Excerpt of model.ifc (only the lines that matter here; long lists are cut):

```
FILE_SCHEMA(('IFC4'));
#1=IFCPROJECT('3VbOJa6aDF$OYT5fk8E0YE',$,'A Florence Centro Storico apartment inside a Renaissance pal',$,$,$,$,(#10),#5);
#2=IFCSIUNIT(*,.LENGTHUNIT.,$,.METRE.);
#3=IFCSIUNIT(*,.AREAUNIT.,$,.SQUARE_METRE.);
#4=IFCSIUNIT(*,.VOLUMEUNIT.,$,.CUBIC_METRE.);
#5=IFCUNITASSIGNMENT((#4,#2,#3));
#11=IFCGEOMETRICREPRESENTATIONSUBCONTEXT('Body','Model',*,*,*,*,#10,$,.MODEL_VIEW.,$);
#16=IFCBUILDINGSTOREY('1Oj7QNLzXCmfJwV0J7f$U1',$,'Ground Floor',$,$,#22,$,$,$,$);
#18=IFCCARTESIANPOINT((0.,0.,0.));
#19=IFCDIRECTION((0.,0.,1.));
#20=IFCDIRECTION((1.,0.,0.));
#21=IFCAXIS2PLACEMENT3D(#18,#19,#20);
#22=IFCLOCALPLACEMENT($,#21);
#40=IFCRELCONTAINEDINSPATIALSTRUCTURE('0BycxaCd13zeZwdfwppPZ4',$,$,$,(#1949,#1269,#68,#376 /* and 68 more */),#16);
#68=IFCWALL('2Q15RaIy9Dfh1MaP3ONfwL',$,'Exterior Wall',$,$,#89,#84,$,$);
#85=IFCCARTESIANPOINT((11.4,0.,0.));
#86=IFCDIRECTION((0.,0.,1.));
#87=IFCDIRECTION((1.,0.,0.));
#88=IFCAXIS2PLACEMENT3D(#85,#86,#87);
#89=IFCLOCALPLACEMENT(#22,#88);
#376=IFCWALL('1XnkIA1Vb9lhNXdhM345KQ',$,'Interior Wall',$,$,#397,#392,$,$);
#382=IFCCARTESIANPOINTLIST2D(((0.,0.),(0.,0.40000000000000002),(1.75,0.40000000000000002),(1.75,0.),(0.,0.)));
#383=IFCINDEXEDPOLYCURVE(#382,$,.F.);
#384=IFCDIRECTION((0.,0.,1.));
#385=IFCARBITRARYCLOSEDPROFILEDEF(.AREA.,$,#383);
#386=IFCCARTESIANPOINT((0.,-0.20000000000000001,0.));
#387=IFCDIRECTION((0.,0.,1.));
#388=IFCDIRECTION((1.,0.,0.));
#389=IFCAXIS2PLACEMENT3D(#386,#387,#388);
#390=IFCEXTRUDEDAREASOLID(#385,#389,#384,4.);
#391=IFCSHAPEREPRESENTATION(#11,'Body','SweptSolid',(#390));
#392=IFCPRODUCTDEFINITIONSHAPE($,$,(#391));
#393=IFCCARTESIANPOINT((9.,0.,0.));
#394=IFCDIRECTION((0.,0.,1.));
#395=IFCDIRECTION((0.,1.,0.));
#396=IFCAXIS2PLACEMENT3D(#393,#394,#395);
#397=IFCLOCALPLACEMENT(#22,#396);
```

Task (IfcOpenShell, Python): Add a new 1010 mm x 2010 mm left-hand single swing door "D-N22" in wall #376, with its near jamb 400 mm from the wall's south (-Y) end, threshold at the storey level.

```python
import numpy as np
import ifcopenshell
import ifcopenshell.api.feature
import ifcopenshell.api.geometry
import ifcopenshell.api.root
import ifcopenshell.api.spatial
import ifcopenshell.geom
import ifcopenshell.util.element
import ifcopenshell.util.placement
import ifcopenshell.util.representation
import ifcopenshell.util.shape
import ifcopenshell.util.unit

model = ifcopenshell.open("model.ifc")
unit_scale = ifcopenshell.util.unit.calculate_unit_scale(model)
settings = ifcopenshell.geom.settings()


def volume(element):
    """Net volume in cubic metres, openings subtracted."""
    shape = ifcopenshell.geom.create_shape(settings, element)
    return ifcopenshell.util.shape.get_volume(shape.geometry)


wall = model.by_guid("1XnkIA1Vb9lhNXdhM345KQ")
storey = ifcopenshell.util.element.get_container(wall, ifc_class="IfcBuildingStorey")
context = ifcopenshell.util.representation.get_context(model, "Model", "Body", "MODEL_VIEW")
before = volume(wall)

width, height, from_end, sill = 1.01, 2.01, 0.4, 0.0  # metres

# The wall runs along its own X axis, and the end named is its -X end.
wall_shape = ifcopenshell.geom.create_shape(settings, wall)
x, y, z = ifcopenshell.util.shape.get_vertices(wall_shape.geometry).T
start = x.min() + from_end
face, thickness = float(y.min()), float(y.max() - y.min())
wall_matrix = ifcopenshell.util.placement.get_local_placement(wall.ObjectPlacement)
level = ifcopenshell.util.placement.get_local_placement(storey.ObjectPlacement)[2, 3]


def in_wall(x, y):
    """Placement at x, y metres in the wall's axes, at sill height."""
    matrix = wall_matrix.copy()
    matrix[:, 3] = wall_matrix @ np.array([x / unit_scale, y / unit_scale, 0.0, 1.0])
    matrix[2, 3] = level + sill / unit_scale
    return matrix


# Opening: a box that overshoots both wall faces by 50 mm.
opening = ifcopenshell.api.root.create_entity(model, ifc_class="IfcOpeningElement", predefined_type="OPENING")
box = ifcopenshell.api.geometry.add_wall_representation(
    model, context=context, length=width, height=height, thickness=thickness + 0.1
)
ifcopenshell.api.geometry.assign_representation(model, product=opening, representation=box)
ifcopenshell.api.geometry.edit_object_placement(model, product=opening, matrix=in_wall(start, face - 0.05), is_si=False)
ifcopenshell.api.feature.add_feature(model, feature=opening, element=wall)

door = ifcopenshell.api.root.create_entity(model, ifc_class="IfcDoor", name="D-N22", predefined_type="DOOR")
door.OverallWidth, door.OverallHeight = width / unit_scale, height / unit_scale
door.OperationType = "SINGLE_SWING_LEFT"
body = ifcopenshell.api.geometry.add_door_representation(
    model,
    context=context,
    overall_width=door.OverallWidth,
    overall_height=door.OverallHeight,
    operation_type="SINGLE_SWING_LEFT",
    lining_properties={"LiningDepth": thickness / unit_scale, "ThresholdDepth": thickness / unit_scale},
)
ifcopenshell.api.geometry.assign_representation(model, product=door, representation=body)
ifcopenshell.api.spatial.assign_container(model, products=[door], relating_structure=storey)
ifcopenshell.api.feature.add_filling(model, opening=opening, element=door)

# The lining spans the wall, so the door starts at the wall face.
ifcopenshell.api.geometry.edit_object_placement(model, product=door, matrix=in_wall(start, face), is_si=False)

after = volume(wall)

print(f"wall volume {before:.3f} -> {after:.3f} m3")

model.write("model_updated.ifc")
```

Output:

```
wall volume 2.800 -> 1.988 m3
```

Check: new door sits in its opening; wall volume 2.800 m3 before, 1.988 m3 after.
